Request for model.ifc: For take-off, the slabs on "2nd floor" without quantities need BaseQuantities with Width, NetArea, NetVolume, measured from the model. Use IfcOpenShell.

First a look at what the model holds.

```python
import ifcopenshell
import ifcopenshell.util.element
import ifcopenshell.util.unit

model = ifcopenshell.open("model.ifc")
print(model.schema)
for unit_type in ("LENGTHUNIT", "AREAUNIT", "VOLUMEUNIT"):
    print(unit_type, ifcopenshell.util.unit.calculate_unit_scale(model, unit_type))
storey = next(s for s in model.by_type("IfcBuildingStorey") if s.Name == "2nd floor")
slabs = [e for e in ifcopenshell.util.element.get_decomposition(storey) if e.is_a("IfcSlab")]
for e in sorted(slabs, key=lambda e: e.id()):
    print(e.id(), e.is_a(), e.Name, list(ifcopenshell.util.element.get_psets(e, qtos_only=True)), sep=" | ")
```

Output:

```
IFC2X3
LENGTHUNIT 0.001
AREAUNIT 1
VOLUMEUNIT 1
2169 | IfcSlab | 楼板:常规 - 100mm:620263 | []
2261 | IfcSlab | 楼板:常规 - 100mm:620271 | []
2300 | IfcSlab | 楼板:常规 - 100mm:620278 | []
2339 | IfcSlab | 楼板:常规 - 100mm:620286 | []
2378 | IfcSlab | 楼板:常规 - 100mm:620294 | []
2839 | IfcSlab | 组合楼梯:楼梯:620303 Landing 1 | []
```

```python
import ifcopenshell
import ifcopenshell.api.pset
import ifcopenshell.geom
import ifcopenshell.util.element
import ifcopenshell.util.shape
import ifcopenshell.util.unit

model = ifcopenshell.open("model.ifc")
unit_scale = ifcopenshell.util.unit.calculate_unit_scale(model)
area_scale = ifcopenshell.util.unit.calculate_unit_scale(model, "AREAUNIT")
volume_scale = ifcopenshell.util.unit.calculate_unit_scale(model, "VOLUMEUNIT")
settings = ifcopenshell.geom.settings()

storey = next(s for s in model.by_type("IfcBuildingStorey") if s.Name == "2nd floor")
slabs = [e for e in ifcopenshell.util.element.get_decomposition(storey) if e.is_a("IfcSlab")]

for e in sorted(slabs, key=lambda e: e.id()):
    if ifcopenshell.util.element.get_psets(e, qtos_only=True, should_inherit=False):
        continue
    # Geometry comes back in metres, in the element's own axes.
    shape = ifcopenshell.geom.create_shape(settings, e)
    values = {
        "Width": ifcopenshell.util.shape.get_z(shape.geometry) / unit_scale,
        "NetArea": ifcopenshell.util.shape.get_footprint_area(shape.geometry) / area_scale,
        "NetVolume": ifcopenshell.util.shape.get_volume(shape.geometry) / volume_scale,
    }
    qto = ifcopenshell.api.pset.add_qto(model, product=e, name="BaseQuantities")
    ifcopenshell.api.pset.edit_qto(model, qto=qto, properties=values)
    print(e.id(), {k: round(v, 3) for k, v in values.items()})

model.write("model_v2.ifc")
```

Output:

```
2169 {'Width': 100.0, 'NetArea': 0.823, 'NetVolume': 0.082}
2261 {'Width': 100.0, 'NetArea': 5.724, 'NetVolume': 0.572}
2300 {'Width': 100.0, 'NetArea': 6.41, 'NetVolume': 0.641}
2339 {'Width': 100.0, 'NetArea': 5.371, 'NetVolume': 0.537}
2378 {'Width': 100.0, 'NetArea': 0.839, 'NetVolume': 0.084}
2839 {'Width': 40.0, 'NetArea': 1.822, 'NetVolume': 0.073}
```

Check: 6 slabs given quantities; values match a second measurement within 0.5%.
